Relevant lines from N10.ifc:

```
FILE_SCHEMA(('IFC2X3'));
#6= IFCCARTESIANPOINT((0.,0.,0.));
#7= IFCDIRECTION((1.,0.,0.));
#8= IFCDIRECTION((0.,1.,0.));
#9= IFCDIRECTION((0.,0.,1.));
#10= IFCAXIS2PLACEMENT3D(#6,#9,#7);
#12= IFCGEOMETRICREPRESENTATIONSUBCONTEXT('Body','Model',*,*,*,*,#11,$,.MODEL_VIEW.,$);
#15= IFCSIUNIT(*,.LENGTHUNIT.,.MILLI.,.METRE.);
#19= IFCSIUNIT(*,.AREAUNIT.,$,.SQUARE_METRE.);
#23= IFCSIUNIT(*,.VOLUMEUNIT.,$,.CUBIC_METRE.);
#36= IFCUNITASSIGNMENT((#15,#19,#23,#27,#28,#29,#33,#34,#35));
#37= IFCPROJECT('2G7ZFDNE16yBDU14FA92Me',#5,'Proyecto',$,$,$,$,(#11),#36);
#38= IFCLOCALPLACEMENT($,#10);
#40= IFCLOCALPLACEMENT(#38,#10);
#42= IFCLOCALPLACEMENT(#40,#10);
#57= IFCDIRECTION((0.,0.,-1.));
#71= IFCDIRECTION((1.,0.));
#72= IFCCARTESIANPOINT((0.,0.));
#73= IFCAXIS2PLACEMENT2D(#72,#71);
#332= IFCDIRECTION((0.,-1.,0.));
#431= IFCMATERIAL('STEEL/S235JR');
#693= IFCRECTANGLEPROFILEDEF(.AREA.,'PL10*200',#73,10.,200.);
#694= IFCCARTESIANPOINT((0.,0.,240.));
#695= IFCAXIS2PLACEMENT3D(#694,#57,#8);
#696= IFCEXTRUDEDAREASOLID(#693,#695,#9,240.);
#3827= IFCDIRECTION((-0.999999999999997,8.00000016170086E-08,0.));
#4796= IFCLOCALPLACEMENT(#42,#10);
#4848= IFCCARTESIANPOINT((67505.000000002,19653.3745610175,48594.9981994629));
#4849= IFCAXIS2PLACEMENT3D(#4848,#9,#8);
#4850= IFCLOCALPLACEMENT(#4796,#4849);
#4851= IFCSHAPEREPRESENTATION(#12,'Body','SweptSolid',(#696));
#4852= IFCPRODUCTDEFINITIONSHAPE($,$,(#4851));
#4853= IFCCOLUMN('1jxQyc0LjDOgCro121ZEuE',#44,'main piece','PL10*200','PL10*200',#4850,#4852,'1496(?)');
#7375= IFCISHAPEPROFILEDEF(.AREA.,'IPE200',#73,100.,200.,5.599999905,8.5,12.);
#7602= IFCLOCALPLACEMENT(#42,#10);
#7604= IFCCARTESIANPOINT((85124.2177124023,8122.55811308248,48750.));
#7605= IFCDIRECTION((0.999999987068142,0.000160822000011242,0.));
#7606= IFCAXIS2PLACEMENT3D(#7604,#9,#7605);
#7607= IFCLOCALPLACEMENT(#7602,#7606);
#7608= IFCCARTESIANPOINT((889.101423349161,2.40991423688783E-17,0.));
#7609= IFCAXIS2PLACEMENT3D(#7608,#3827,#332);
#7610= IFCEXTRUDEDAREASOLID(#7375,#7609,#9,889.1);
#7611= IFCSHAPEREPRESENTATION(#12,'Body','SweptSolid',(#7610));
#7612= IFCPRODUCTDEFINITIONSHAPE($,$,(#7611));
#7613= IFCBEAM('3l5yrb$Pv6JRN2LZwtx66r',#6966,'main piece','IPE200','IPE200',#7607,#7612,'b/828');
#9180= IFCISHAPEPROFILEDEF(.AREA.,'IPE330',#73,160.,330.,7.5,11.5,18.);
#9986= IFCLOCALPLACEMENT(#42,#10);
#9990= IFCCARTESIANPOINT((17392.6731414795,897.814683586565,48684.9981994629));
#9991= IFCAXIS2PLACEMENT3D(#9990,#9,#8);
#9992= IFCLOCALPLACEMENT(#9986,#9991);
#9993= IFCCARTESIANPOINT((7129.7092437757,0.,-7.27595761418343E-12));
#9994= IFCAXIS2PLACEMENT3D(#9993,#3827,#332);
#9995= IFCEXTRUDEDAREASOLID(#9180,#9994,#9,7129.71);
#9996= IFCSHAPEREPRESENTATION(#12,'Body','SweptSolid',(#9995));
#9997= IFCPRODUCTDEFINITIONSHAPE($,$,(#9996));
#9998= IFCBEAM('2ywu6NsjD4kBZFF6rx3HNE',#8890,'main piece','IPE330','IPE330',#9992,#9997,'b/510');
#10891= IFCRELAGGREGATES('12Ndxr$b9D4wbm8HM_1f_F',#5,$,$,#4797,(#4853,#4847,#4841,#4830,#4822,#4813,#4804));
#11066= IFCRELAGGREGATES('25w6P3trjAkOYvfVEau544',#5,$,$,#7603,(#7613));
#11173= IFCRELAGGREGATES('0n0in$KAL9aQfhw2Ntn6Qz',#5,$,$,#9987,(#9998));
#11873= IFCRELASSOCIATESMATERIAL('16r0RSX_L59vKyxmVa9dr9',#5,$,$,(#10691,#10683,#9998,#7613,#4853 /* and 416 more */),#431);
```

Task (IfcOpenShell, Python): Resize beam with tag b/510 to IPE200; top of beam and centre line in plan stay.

```python
import ifcopenshell
import ifcopenshell.util.element
import ifcopenshell.util.representation

model = ifcopenshell.open("N10.ifc")

member = model.by_id(9998)
source = next(p for p in model.by_type("IfcIShapeProfileDef") if p.ProfileName == "IPE200")

body = ifcopenshell.util.representation.get_representation(member, "Model", "Body")
solid = body.Items[0]
old_profile = solid.SweptArea

# Copy the section's sizes but keep this member's own profile position.
profile = ifcopenshell.util.element.copy(model, source)
# Profiles are centred, so shift by half the change in depth to hold the top.
shift = (old_profile.OverallDepth - profile.OverallDepth) / 2
x, y = old_profile.Position.Location.Coordinates
up = (0.0, 1.0)  # upwards, in the solid's own plane
location = model.createIfcCartesianPoint((x + up[0] * shift, y + up[1] * shift))
profile.Position = model.createIfcAxis2Placement2D(location, old_profile.Position.RefDirection)
solid.SweptArea = profile
if not model.get_total_inverses(old_profile):
    ifcopenshell.util.element.remove_deep2(model, old_profile)
member.Description = member.Description.replace("IPE330", "IPE200")
member.ObjectType = member.ObjectType.replace("IPE330", "IPE200")

print(solid.SweptArea)

model.write("N10_updated.ifc")
```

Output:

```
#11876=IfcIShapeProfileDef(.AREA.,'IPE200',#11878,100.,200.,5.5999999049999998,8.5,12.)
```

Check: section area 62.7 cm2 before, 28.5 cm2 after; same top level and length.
